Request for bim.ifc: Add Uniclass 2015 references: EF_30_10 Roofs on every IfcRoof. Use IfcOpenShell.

First a look at what the model holds.

```python
import ifcopenshell

model = ifcopenshell.open("bim.ifc")
print(model.schema)
print("classifications:", [c.Name for c in model.by_type("IfcClassification")])
for ifc_class in ("IfcDoor", "IfcRoof", "IfcStair", "IfcWall", "IfcWindow"):
    print(ifc_class, len(model.by_type(ifc_class)))
```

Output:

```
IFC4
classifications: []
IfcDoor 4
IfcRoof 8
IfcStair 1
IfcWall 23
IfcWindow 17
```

```python
import ifcopenshell
import ifcopenshell.api.classification

model = ifcopenshell.open("bim.ifc")

system = ifcopenshell.api.classification.add_classification(model, classification="Uniclass 2015")

codes = {
    "IfcRoof": ("EF_30_10", "Roofs"),
}
for ifc_class, (code, name) in codes.items():
    products = model.by_type(ifc_class)
    ifcopenshell.api.classification.add_reference(
        model, products=products, classification=system, identification=code, name=name
    )
    print(code, len(products))

model.write("bim_updated.ifc")
```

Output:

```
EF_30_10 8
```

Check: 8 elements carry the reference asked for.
